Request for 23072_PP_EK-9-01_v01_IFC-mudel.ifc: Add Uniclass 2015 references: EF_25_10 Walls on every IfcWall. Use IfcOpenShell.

First a look at what the model holds.

```python
import ifcopenshell

model = ifcopenshell.open("23072_PP_EK-9-01_v01_IFC-mudel.ifc")
print(model.schema)
print("classifications:", [c.Name for c in model.by_type("IfcClassification")])
for ifc_class in ("IfcDoor", "IfcRoof", "IfcStair", "IfcWall", "IfcWindow"):
    print(ifc_class, len(model.by_type(ifc_class)))
```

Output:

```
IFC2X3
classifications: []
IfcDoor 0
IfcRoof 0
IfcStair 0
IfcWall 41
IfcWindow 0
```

```python
import ifcopenshell
import ifcopenshell.api.classification

model = ifcopenshell.open("23072_PP_EK-9-01_v01_IFC-mudel.ifc")

# IFC2X3 requires Source and Edition and has no link from the project to the system.
system = model.create_entity("IfcClassification", Source="NBS", Edition="2015", Name="Uniclass 2015")

codes = {
    "IfcWall": ("EF_25_10", "Walls"),
}
for ifc_class, (code, name) in codes.items():
    products = model.by_type(ifc_class)
    ifcopenshell.api.classification.add_reference(
        model, products=products, classification=system, identification=code, name=name
    )
    print(code, len(products))

model.write("23072_PP_EK-9-01_v01_IFC-mudel_v2.ifc")
```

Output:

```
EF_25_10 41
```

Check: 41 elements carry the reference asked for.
